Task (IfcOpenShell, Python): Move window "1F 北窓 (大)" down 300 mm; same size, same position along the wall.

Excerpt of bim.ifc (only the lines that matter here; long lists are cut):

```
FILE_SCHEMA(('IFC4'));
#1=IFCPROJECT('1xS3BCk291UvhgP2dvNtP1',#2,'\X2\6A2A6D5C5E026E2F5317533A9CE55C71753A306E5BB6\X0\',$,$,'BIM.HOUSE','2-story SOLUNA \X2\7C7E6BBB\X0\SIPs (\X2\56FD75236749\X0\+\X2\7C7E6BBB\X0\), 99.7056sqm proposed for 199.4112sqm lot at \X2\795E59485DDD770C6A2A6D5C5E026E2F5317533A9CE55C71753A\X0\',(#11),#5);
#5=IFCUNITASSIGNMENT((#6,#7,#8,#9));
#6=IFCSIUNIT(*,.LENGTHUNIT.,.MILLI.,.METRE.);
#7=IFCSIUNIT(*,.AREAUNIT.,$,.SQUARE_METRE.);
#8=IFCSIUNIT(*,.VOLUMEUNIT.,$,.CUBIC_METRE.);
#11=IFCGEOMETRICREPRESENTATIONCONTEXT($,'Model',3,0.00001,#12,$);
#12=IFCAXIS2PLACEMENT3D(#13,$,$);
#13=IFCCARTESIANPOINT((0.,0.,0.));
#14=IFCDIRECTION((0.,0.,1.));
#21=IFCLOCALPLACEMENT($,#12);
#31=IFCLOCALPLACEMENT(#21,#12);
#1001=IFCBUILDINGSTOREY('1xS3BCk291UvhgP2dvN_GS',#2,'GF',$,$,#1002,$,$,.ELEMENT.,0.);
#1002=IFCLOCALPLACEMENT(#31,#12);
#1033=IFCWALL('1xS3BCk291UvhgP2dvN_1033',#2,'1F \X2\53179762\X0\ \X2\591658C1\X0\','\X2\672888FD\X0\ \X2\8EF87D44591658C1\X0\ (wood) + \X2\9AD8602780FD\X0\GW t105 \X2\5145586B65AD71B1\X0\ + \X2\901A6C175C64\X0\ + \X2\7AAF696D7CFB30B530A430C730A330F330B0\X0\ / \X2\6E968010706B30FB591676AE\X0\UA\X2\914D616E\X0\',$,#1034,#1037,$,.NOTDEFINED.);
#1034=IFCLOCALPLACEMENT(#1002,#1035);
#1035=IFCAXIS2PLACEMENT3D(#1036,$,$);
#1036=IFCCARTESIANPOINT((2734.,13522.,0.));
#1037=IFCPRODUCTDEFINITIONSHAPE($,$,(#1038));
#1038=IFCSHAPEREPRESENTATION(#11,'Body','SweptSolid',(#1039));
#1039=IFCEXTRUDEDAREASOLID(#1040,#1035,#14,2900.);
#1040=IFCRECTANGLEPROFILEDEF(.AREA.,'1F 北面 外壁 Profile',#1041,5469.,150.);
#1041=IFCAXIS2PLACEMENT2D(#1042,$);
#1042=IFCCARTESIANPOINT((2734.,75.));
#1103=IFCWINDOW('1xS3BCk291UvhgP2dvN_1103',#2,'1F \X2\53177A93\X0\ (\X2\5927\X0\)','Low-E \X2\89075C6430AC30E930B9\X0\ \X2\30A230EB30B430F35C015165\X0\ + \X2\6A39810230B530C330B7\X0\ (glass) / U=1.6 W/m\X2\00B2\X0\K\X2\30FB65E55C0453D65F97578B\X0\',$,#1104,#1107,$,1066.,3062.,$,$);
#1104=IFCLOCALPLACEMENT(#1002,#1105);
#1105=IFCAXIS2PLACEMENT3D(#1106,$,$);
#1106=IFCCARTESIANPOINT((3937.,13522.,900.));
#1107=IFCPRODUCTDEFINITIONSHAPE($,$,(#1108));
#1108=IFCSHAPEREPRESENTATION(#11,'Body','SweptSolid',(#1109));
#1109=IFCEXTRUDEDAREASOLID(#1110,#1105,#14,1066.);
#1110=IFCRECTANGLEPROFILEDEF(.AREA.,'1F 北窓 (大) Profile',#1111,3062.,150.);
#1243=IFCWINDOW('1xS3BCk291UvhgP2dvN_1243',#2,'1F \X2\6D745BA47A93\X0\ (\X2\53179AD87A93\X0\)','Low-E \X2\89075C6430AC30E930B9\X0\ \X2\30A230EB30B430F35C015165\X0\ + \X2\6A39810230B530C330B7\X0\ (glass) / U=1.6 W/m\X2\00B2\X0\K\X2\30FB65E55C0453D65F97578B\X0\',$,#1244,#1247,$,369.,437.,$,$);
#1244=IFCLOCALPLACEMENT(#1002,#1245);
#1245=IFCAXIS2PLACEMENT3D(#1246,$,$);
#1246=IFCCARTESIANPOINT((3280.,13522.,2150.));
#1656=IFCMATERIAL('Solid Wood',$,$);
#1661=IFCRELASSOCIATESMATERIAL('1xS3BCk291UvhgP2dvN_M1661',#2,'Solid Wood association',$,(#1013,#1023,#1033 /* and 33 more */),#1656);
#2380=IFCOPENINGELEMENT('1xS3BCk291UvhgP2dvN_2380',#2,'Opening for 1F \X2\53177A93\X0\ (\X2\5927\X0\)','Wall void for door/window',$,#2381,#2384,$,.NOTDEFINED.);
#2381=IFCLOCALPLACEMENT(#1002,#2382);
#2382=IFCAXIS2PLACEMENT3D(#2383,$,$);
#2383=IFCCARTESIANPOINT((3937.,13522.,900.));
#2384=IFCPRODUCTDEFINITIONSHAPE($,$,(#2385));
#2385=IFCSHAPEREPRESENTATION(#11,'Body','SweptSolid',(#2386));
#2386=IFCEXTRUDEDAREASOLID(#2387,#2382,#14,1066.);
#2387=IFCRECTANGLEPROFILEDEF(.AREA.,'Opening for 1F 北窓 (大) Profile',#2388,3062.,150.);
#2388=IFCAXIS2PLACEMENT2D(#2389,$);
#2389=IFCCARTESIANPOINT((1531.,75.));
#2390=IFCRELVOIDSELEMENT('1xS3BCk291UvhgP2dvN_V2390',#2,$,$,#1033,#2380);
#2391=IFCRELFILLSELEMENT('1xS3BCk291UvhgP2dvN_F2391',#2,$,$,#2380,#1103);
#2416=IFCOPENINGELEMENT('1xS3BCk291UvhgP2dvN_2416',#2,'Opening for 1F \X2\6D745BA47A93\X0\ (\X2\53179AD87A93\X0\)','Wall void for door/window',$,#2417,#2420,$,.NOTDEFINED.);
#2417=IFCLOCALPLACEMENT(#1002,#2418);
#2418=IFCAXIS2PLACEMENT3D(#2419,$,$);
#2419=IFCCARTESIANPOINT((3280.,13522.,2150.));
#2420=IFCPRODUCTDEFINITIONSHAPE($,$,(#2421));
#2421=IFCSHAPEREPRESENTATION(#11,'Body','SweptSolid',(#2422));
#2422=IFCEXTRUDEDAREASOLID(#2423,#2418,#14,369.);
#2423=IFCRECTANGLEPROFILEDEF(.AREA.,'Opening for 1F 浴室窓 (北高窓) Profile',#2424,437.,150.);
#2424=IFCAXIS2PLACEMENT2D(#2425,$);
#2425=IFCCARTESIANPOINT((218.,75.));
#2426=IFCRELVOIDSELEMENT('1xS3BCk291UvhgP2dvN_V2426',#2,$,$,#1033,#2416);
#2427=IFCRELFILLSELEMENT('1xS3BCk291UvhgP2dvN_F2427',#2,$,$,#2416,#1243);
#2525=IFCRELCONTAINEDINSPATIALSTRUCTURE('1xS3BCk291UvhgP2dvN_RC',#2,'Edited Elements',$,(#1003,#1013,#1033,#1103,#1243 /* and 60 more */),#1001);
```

```python
import numpy as np
import ifcopenshell
import ifcopenshell.api.geometry
import ifcopenshell.util.placement
import ifcopenshell.util.unit

model = ifcopenshell.open("bim.ifc")
unit_scale = ifcopenshell.util.unit.calculate_unit_scale(model)

window = model.by_guid("1xS3BCk291UvhgP2dvN_1103")
opening = window.FillsVoids[0].RelatingOpeningElement
dz = -300.0

shift = np.array([0.0, 0.0, dz])
# The window is not placed relative to its opening, so move both.
for product in (opening, window):
    matrix = ifcopenshell.util.placement.get_local_placement(product.ObjectPlacement)
    matrix[:3, 3] += shift
    ifcopenshell.api.geometry.edit_object_placement(model, product=product, matrix=matrix, is_si=False)

print(f"moved by {dz * unit_scale:+.3f} m")

model.write("bim_v2.ifc")
```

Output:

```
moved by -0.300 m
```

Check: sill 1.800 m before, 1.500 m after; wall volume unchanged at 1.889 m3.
